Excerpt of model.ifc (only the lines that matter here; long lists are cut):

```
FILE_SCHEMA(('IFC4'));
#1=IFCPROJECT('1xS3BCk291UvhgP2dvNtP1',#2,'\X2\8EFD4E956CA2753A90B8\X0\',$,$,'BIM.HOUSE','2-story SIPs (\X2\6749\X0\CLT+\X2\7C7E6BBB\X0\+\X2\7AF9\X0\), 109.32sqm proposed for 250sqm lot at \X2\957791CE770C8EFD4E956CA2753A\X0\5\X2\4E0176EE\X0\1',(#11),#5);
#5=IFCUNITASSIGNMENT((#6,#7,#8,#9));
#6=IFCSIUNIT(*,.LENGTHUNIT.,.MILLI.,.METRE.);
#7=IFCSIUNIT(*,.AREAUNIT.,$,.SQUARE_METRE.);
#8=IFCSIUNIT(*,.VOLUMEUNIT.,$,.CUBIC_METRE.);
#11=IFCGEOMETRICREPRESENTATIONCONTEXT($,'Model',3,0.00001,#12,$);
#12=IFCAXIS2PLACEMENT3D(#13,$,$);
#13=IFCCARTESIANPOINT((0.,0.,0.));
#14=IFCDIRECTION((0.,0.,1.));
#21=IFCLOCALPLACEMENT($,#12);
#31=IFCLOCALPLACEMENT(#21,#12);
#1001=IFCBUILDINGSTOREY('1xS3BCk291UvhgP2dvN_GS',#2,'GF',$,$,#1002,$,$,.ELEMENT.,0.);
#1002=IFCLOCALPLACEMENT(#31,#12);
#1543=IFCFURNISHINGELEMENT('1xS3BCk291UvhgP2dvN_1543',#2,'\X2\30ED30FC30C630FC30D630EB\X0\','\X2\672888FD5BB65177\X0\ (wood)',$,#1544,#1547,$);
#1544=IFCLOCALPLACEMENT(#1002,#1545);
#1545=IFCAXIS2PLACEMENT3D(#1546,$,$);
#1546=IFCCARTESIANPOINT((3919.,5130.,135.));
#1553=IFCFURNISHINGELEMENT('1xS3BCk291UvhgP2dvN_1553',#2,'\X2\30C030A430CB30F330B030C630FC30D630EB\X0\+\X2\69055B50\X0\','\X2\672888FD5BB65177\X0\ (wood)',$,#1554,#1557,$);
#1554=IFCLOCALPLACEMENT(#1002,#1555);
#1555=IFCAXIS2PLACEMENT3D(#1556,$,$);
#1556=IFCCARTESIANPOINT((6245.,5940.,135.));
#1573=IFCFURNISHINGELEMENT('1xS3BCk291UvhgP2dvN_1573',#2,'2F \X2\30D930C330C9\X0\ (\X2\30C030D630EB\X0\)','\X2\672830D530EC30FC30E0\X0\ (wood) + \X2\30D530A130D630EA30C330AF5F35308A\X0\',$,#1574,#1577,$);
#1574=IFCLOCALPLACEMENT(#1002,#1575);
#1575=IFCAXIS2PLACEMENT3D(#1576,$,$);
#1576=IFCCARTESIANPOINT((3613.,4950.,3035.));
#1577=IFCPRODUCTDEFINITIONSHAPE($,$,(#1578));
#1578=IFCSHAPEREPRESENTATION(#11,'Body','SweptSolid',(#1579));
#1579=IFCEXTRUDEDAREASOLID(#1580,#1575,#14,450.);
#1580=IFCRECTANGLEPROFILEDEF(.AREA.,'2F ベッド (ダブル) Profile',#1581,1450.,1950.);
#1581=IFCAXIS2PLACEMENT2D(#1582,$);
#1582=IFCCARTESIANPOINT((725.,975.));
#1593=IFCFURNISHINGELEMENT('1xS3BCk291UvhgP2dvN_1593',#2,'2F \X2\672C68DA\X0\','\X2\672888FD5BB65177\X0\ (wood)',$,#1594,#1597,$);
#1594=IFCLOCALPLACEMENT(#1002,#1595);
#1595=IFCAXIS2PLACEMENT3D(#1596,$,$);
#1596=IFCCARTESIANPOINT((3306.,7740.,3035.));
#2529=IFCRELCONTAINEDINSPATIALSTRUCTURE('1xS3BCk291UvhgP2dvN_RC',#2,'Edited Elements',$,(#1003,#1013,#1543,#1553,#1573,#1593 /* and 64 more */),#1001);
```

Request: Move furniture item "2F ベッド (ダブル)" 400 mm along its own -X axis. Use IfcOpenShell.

```python
import ifcopenshell
import ifcopenshell.api.geometry
import ifcopenshell.util.placement
import ifcopenshell.util.unit

model = ifcopenshell.open("model.ifc")
unit_scale = ifcopenshell.util.unit.calculate_unit_scale(model)

item = model.by_guid("1xS3BCk291UvhgP2dvN_1573")
matrix = ifcopenshell.util.placement.get_local_placement(item.ObjectPlacement)
matrix[:3, 3] -= matrix[:3, 0] * 0.4 / unit_scale
ifcopenshell.api.geometry.edit_object_placement(model, product=item, matrix=matrix, is_si=False)

print(ifcopenshell.util.placement.get_local_placement(item.ObjectPlacement).round(3) + 0.0)

model.write("model_rev.ifc")
```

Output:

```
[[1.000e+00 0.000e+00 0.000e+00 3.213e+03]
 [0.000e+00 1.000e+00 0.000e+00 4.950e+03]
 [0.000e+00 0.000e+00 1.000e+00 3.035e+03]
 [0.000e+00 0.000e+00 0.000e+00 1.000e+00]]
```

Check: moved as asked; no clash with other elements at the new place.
